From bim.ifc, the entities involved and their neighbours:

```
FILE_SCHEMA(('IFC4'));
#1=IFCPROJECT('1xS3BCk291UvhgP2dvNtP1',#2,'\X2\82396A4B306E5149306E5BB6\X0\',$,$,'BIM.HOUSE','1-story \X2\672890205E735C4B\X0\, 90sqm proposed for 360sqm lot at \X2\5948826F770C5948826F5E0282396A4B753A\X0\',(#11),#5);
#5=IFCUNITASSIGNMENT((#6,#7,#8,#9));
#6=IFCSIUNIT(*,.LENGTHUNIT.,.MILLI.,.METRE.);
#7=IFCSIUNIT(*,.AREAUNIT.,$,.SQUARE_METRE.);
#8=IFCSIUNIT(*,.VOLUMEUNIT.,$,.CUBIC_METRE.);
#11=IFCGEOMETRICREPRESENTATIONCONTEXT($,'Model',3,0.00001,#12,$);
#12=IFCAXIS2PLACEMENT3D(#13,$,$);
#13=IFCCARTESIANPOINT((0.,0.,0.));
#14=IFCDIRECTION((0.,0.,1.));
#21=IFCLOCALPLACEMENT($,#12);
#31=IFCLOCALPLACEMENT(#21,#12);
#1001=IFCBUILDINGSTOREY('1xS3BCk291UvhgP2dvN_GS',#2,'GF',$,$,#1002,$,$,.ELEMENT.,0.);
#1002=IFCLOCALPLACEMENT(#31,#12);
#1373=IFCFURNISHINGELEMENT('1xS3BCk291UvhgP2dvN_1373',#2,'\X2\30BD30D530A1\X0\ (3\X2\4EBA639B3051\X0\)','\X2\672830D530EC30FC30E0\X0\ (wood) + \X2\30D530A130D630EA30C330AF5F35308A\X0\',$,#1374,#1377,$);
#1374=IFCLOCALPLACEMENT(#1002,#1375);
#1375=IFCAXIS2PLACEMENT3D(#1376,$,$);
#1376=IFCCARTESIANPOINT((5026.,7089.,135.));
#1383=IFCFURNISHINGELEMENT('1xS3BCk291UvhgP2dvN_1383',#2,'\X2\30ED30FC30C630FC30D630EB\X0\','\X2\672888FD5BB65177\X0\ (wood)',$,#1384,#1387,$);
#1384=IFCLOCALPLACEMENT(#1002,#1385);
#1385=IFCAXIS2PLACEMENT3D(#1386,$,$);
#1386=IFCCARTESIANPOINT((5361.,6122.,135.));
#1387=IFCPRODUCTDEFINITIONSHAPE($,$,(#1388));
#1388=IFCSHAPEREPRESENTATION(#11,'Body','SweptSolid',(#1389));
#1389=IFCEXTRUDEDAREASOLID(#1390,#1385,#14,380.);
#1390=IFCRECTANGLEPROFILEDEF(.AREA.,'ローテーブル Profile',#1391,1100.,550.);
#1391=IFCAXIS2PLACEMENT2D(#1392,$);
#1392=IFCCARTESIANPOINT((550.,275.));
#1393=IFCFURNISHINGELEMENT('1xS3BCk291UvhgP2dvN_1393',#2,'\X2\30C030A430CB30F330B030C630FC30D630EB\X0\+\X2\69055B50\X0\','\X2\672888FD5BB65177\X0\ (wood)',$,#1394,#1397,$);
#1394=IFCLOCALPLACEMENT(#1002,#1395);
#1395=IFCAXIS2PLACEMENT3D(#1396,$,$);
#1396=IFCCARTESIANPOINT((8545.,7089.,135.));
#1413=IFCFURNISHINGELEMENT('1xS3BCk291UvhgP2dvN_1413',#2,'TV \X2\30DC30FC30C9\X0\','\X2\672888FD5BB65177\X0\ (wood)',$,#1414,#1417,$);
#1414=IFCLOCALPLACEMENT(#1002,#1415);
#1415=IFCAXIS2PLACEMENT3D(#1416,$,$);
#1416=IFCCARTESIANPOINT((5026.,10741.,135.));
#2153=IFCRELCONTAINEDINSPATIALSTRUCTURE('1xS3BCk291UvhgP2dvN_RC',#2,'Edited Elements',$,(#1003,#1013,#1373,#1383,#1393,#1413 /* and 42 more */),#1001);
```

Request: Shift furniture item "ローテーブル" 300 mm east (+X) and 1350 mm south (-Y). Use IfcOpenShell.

```python
import ifcopenshell
import ifcopenshell.api.geometry
import ifcopenshell.util.placement
import ifcopenshell.util.unit

model = ifcopenshell.open("bim.ifc")
unit_scale = ifcopenshell.util.unit.calculate_unit_scale(model)

item = model.by_guid("1xS3BCk291UvhgP2dvN_1383")
matrix = ifcopenshell.util.placement.get_local_placement(item.ObjectPlacement)
matrix[0, 3] += 0.3 / unit_scale
matrix[1, 3] -= 1.35 / unit_scale
ifcopenshell.api.geometry.edit_object_placement(model, product=item, matrix=matrix, is_si=False)

print(ifcopenshell.util.placement.get_local_placement(item.ObjectPlacement).round(3) + 0.0)

model.write("bim-out.ifc")
```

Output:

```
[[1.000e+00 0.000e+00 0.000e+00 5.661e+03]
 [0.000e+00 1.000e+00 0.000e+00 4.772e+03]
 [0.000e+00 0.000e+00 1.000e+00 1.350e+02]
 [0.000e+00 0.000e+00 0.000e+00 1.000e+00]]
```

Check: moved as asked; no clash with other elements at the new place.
